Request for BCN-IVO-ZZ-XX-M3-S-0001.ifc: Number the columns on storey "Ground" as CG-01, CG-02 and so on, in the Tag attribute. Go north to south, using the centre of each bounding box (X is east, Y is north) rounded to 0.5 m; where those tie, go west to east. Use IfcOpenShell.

First a look at what the model holds.

```python
import ifcopenshell
import ifcopenshell.util.element
import ifcopenshell.util.placement

model = ifcopenshell.open("BCN-IVO-ZZ-XX-M3-S-0001.ifc")
print(model.schema)
storey = next(s for s in model.by_type("IfcBuildingStorey") if s.Name == "Ground")
columns = [e for e in ifcopenshell.util.element.get_decomposition(storey) if e.is_a("IfcColumn")]
for e in sorted(columns, key=lambda e: e.id()):
    origin = ifcopenshell.util.placement.get_local_placement(e.ObjectPlacement)[:3, 3]
    print(e.id(), e.Tag, e.Name, origin.round(2) + 0.0, sep=" | ")
```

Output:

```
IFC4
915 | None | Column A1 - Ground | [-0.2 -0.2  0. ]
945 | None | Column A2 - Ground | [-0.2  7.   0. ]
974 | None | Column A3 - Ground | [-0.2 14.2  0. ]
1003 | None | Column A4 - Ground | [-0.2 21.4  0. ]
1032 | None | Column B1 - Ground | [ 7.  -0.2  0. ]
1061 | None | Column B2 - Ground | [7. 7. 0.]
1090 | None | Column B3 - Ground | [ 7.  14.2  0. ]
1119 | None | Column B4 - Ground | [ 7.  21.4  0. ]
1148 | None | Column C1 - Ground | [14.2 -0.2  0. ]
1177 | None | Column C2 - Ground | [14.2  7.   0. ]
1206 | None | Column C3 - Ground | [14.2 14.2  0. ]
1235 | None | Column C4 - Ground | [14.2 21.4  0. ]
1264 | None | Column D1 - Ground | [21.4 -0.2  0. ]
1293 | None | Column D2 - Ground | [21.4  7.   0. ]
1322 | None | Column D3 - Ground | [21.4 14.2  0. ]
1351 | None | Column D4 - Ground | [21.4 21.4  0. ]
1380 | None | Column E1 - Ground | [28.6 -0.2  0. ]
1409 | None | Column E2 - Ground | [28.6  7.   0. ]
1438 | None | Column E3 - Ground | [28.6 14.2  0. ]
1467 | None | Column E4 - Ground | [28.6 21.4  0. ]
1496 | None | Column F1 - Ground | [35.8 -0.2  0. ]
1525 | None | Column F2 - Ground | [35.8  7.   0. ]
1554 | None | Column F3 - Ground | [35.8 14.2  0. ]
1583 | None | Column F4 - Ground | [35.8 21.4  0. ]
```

```python
import ifcopenshell
import ifcopenshell.geom
import ifcopenshell.util.element
import ifcopenshell.util.shape

model = ifcopenshell.open("BCN-IVO-ZZ-XX-M3-S-0001.ifc")
settings = ifcopenshell.geom.settings()
settings.set("use-world-coords", True)


def centre(element):
    shape = ifcopenshell.geom.create_shape(settings, element)
    return ifcopenshell.util.shape.get_bbox_centroid(shape.geometry)


storey = next(s for s in model.by_type("IfcBuildingStorey") if s.Name == "Ground")
columns = [e for e in ifcopenshell.util.element.get_decomposition(storey) if e.is_a("IfcColumn")]

# Insertion points can sit at a corner or the storey origin, so sort by the geometry (in metres).
centres = {e: centre(e) for e in columns}
columns.sort(key=lambda e: (-round(centres[e][1] / 0.5), centres[e][0]))

for i, e in enumerate(columns, start=1):
    number = f"CG-{i:02d}"
    e.Tag = number
    print(e.id(), number)

model.write("BCN-IVO-ZZ-XX-M3-S-0001_updated.ifc")
```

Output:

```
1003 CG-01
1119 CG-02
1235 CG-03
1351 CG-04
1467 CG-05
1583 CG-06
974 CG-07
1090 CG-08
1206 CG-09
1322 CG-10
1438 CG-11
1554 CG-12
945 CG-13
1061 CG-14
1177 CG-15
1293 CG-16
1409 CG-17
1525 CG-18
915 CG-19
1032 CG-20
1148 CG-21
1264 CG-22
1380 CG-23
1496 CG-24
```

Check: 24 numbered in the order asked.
